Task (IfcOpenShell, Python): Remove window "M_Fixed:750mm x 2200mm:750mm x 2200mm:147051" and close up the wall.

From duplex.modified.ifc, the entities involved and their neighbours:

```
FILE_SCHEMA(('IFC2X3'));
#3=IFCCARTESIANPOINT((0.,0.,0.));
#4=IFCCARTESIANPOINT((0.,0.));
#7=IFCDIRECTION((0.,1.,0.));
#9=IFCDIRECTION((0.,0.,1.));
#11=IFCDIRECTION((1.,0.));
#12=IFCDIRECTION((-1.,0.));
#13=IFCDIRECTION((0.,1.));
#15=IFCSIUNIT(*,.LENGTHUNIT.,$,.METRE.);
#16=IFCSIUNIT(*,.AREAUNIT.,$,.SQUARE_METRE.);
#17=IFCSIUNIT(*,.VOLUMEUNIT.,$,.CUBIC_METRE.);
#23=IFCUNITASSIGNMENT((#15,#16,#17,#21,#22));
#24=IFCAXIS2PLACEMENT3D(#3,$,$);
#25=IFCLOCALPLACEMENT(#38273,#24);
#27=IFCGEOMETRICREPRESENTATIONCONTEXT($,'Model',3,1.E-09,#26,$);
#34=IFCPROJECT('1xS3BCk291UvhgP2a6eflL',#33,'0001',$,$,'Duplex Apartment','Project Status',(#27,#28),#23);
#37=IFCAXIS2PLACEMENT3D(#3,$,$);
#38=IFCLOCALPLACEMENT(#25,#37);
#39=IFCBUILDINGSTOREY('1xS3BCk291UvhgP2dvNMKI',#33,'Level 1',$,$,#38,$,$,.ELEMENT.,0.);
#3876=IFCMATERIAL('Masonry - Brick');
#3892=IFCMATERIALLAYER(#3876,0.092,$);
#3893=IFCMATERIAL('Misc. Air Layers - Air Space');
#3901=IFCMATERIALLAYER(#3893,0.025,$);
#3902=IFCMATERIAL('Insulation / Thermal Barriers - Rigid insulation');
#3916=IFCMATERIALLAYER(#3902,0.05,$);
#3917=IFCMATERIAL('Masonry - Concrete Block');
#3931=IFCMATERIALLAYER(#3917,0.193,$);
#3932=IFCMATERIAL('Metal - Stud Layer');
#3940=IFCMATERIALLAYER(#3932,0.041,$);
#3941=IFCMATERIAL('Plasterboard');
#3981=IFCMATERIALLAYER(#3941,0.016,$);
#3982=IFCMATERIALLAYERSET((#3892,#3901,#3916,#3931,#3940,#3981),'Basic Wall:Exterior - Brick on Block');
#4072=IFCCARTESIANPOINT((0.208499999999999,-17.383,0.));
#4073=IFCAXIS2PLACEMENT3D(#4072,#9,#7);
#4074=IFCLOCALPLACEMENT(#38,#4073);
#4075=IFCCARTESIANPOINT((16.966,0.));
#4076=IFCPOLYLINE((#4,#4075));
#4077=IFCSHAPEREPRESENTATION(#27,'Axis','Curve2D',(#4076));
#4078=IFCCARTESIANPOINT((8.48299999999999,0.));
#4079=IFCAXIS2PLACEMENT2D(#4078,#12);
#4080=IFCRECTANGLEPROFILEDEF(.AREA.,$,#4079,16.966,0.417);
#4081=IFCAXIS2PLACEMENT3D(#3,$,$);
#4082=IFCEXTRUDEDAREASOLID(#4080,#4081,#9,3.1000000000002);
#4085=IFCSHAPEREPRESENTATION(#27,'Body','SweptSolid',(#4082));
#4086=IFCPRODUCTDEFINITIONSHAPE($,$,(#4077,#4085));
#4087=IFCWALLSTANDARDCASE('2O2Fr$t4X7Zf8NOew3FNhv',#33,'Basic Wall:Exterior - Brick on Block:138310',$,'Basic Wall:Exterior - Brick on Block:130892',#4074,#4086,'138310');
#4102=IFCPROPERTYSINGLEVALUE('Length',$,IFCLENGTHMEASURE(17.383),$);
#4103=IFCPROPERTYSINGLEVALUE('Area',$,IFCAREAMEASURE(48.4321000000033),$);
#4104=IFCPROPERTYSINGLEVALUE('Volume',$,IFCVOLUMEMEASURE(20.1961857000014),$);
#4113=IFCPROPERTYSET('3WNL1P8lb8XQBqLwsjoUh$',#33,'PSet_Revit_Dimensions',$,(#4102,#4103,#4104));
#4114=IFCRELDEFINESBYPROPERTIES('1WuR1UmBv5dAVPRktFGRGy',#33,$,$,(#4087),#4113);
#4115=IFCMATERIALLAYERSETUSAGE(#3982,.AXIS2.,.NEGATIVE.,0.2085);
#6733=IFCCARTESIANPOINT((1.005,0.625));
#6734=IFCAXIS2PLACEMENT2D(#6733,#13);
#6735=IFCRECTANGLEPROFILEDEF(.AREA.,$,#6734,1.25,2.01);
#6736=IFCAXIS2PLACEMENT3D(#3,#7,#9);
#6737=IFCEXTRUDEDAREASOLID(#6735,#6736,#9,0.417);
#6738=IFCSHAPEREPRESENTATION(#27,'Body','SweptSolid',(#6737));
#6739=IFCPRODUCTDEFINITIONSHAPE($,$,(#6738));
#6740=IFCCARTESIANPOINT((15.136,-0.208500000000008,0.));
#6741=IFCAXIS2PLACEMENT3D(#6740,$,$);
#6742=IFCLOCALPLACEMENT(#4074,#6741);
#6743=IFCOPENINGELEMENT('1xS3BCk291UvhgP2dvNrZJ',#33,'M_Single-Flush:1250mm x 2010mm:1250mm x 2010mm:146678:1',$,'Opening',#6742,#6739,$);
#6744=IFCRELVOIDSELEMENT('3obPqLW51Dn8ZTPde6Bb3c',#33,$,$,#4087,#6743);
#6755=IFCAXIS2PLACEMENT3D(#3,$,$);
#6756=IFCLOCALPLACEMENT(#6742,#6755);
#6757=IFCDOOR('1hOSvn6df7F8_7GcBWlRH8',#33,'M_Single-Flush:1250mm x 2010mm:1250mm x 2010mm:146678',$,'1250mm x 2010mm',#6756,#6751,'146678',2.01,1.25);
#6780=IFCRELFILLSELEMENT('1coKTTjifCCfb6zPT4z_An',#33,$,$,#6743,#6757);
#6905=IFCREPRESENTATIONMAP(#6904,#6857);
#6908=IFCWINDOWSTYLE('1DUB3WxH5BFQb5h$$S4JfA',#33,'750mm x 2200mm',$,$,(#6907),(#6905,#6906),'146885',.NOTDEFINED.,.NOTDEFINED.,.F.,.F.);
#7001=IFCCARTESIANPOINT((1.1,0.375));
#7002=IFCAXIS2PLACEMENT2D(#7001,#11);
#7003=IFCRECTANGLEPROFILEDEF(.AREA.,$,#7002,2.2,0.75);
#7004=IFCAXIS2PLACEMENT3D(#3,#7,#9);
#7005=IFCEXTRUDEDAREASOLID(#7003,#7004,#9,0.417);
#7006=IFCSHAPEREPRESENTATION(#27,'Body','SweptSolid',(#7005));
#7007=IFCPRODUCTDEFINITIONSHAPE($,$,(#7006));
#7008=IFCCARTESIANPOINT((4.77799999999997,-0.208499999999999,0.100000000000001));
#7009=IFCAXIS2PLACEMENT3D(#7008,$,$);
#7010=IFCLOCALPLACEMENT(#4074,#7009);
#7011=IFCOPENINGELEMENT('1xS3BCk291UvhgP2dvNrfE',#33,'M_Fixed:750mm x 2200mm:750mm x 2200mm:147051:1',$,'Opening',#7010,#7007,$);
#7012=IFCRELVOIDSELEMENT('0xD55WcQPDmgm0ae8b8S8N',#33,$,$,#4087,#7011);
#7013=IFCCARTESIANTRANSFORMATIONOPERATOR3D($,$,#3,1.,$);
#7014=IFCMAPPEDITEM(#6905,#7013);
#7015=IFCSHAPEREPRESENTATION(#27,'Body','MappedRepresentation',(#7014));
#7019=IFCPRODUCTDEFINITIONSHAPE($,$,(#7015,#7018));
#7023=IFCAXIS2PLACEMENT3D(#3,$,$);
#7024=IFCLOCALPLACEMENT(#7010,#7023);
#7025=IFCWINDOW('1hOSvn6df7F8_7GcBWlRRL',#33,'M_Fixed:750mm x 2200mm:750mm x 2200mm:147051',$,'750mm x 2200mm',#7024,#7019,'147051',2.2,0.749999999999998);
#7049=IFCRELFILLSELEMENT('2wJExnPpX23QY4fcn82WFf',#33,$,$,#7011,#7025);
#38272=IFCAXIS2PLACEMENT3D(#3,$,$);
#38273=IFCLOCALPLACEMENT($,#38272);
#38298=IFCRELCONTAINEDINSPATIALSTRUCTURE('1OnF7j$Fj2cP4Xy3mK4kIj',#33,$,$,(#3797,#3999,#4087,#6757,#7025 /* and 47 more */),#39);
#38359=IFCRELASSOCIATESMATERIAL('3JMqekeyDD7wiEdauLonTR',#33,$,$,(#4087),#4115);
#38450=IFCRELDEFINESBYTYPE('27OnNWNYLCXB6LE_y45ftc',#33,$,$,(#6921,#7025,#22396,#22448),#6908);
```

```python
import ifcopenshell
import ifcopenshell.api.feature
import ifcopenshell.api.pset
import ifcopenshell.api.root
import ifcopenshell.geom
import ifcopenshell.util.element
import ifcopenshell.util.shape
import ifcopenshell.util.unit

model = ifcopenshell.open("duplex.modified.ifc")
area_scale = ifcopenshell.util.unit.calculate_unit_scale(model, "AREAUNIT")
volume_scale = ifcopenshell.util.unit.calculate_unit_scale(model, "VOLUMEUNIT")
settings = ifcopenshell.geom.settings()


def volume(element):
    """Net volume in cubic metres, openings subtracted."""
    shape = ifcopenshell.geom.create_shape(settings, element)
    return ifcopenshell.util.shape.get_volume(shape.geometry)


window = model.by_guid("1hOSvn6df7F8_7GcBWlRRL")
opening = window.FillsVoids[0].RelatingOpeningElement
wall = opening.VoidsElements[0].RelatingBuildingElement
before = volume(wall)

ifcopenshell.api.root.remove_product(model, product=window)
ifcopenshell.api.feature.remove_feature(model, feature=opening)

after = volume(wall)
thickness = 0.417  # wall thickness in metres

# Update the wall's stored quantities.
pset = model.by_id(ifcopenshell.util.element.get_pset(wall, "PSet_Revit_Dimensions", should_inherit=False)["id"])
ifcopenshell.api.pset.edit_pset(model, pset=pset, properties={
    "Area": model.create_entity("IfcAreaMeasure", after / thickness / area_scale),
    "Volume": model.create_entity("IfcVolumeMeasure", after / volume_scale),
})

print(f"wall volume {before:.3f} -> {after:.3f} m3")

model.write("duplex.modified_rev.ifc")
```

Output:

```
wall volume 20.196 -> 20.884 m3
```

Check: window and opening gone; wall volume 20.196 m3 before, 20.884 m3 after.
